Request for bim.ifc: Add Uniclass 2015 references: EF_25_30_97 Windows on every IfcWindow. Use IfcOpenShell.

First a look at what the model holds.

```python
import ifcopenshell

model = ifcopenshell.open("bim.ifc")
print(model.schema)
print("classifications:", [c.Name for c in model.by_type("IfcClassification")])
for ifc_class in ("IfcDoor", "IfcRoof", "IfcStair", "IfcWall", "IfcWindow"):
    print(ifc_class, len(model.by_type(ifc_class)))
```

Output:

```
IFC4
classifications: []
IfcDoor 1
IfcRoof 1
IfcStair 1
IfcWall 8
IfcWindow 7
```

```python
import ifcopenshell
import ifcopenshell.api.classification

model = ifcopenshell.open("bim.ifc")

system = ifcopenshell.api.classification.add_classification(model, classification="Uniclass 2015")

codes = {
    "IfcWindow": ("EF_25_30_97", "Windows"),
}
for ifc_class, (code, name) in codes.items():
    products = model.by_type(ifc_class)
    ifcopenshell.api.classification.add_reference(
        model, products=products, classification=system, identification=code, name=name
    )
    print(code, len(products))

model.write("bim_edited.ifc")
```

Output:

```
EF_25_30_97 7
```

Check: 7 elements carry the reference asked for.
